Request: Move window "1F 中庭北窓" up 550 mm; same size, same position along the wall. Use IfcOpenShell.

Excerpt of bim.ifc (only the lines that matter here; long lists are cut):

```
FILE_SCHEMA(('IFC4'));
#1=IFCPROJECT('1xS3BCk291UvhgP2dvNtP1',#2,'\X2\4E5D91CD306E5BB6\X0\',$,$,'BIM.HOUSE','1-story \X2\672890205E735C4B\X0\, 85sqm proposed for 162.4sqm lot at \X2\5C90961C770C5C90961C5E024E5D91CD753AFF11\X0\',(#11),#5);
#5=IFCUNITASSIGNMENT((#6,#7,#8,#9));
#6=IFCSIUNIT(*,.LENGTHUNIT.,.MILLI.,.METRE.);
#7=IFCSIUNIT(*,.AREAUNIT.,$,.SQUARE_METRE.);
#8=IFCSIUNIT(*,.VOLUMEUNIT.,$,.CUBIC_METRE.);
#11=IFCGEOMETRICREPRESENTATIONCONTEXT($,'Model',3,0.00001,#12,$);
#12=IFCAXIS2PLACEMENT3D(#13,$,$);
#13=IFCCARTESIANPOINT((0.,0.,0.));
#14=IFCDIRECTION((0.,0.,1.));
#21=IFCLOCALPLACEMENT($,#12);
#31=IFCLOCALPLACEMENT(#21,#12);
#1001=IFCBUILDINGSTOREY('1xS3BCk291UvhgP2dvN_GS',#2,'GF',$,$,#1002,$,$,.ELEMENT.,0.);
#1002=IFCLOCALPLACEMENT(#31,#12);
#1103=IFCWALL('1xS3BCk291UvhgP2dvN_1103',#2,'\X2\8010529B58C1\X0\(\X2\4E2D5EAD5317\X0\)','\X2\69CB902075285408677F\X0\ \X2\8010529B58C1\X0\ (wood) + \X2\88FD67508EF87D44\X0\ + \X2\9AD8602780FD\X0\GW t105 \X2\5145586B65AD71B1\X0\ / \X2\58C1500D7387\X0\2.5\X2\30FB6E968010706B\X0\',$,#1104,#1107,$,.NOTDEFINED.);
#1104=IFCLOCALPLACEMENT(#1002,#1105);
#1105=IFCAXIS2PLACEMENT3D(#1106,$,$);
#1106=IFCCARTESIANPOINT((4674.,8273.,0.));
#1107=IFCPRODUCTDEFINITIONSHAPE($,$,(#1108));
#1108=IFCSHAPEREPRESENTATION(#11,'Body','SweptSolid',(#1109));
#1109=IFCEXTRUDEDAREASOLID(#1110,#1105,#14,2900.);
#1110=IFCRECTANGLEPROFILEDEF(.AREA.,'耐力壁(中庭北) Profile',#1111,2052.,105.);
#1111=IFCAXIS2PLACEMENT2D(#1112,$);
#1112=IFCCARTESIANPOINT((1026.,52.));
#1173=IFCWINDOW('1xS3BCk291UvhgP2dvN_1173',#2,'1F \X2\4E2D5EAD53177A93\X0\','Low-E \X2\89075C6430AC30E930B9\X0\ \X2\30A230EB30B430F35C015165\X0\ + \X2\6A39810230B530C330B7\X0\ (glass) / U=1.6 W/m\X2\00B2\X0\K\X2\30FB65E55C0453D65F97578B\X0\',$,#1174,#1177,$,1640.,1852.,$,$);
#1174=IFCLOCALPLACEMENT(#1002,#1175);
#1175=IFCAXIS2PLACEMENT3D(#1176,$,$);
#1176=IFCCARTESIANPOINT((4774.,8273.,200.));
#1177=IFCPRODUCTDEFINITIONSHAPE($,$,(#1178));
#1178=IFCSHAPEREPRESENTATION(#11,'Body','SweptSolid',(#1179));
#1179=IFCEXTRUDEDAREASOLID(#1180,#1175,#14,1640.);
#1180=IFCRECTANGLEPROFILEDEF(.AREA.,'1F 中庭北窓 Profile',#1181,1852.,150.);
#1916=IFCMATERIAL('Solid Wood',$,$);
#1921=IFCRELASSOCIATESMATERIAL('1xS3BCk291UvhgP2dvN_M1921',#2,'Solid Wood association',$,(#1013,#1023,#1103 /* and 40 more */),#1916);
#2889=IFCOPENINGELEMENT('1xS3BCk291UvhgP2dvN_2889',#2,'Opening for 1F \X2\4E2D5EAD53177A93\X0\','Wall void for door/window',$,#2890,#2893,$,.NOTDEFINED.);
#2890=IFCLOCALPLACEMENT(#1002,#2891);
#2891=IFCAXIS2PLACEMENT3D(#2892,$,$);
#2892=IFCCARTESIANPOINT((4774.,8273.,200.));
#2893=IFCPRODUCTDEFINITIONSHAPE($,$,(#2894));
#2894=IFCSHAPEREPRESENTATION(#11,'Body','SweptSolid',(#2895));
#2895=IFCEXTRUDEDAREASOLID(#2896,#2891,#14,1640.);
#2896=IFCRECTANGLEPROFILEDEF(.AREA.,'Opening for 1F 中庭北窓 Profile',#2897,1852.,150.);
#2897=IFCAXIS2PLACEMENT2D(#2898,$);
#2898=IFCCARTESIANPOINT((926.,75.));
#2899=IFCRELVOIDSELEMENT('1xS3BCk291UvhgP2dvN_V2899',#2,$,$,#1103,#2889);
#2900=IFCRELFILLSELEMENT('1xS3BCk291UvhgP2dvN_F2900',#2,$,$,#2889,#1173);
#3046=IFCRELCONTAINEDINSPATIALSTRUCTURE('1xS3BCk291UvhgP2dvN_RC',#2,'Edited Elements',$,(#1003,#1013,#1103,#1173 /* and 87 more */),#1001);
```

```python
import numpy as np
import ifcopenshell
import ifcopenshell.api.geometry
import ifcopenshell.util.placement
import ifcopenshell.util.unit

model = ifcopenshell.open("bim.ifc")
unit_scale = ifcopenshell.util.unit.calculate_unit_scale(model)

window = model.by_guid("1xS3BCk291UvhgP2dvN_1173")
opening = window.FillsVoids[0].RelatingOpeningElement
dz = 0.55 / unit_scale

shift = np.array([0.0, 0.0, dz])
# The window is not placed relative to its opening, so move both.
for product in (opening, window):
    matrix = ifcopenshell.util.placement.get_local_placement(product.ObjectPlacement)
    matrix[:3, 3] += shift
    ifcopenshell.api.geometry.edit_object_placement(model, product=product, matrix=matrix, is_si=False)

print(f"moved by {dz * unit_scale:+.3f} m")

model.write("bim_rev.ifc")
```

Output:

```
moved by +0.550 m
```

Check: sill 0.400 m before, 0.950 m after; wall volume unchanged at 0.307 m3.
